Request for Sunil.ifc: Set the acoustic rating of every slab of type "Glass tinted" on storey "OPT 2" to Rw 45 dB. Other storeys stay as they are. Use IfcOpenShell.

First a look at what the model holds.

```python
import ifcopenshell
import ifcopenshell.util.element

model = ifcopenshell.open("Sunil.ifc")
print(model.schema)
storey = next(s for s in model.by_type("IfcBuildingStorey") if s.Name == "OPT 2")
slabs = [e for e in ifcopenshell.util.element.get_decomposition(storey) if e.is_a("IfcSlab")]
seen = {}
for e in slabs:
    element_type = ifcopenshell.util.element.get_type(e)
    key = (element_type.Name if element_type != e and element_type else None, ifcopenshell.util.element.get_pset(e, "Pset_SlabCommon", "AcousticRating"))
    seen[key] = seen.get(key, 0) + 1
for (name, value), count in sorted(seen.items(), key=str):
    print(count, "x", name, "|", value)
```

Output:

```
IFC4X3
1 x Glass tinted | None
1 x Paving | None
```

```python
import ifcopenshell
import ifcopenshell.api.pset
import ifcopenshell.util.element

model = ifcopenshell.open("Sunil.ifc")

storey = next(s for s in model.by_type("IfcBuildingStorey") if s.Name == "OPT 2")
slabs = [e for e in ifcopenshell.util.element.get_decomposition(storey) if e.is_a("IfcSlab")]

count = 0
for e in slabs:
    element_type = ifcopenshell.util.element.get_type(e)
    if element_type in (None, e) or element_type.Name != "Glass tinted":
        continue
    # add_pset returns the element's existing set when there is one.
    pset = ifcopenshell.api.pset.add_pset(model, product=e, name="Pset_SlabCommon")
    ifcopenshell.api.pset.edit_pset(model, pset=pset, properties={"AcousticRating": "Rw 45 dB"})
    count += 1

print(count, "slabs updated")

model.write("Sunil_v2.ifc")
```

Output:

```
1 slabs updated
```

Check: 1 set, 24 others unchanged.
